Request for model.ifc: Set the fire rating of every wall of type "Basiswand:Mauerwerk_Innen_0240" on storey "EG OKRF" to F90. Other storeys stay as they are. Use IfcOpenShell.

First a look at what the model holds.

```python
import ifcopenshell
import ifcopenshell.util.element

model = ifcopenshell.open("model.ifc")
print(model.schema)
storey = next(s for s in model.by_type("IfcBuildingStorey") if s.Name == "EG OKRF")
walls = [e for e in ifcopenshell.util.element.get_decomposition(storey) if e.is_a("IfcWall")]
seen = {}
for e in walls:
    element_type = ifcopenshell.util.element.get_type(e)
    key = (element_type.Name if element_type != e and element_type else None, ifcopenshell.util.element.get_pset(e, "Pset_WallCommon", "FireRating"))
    seen[key] = seen.get(key, 0) + 1
for (name, value), count in sorted(seen.items(), key=str):
    print(count, "x", name, "|", value)
```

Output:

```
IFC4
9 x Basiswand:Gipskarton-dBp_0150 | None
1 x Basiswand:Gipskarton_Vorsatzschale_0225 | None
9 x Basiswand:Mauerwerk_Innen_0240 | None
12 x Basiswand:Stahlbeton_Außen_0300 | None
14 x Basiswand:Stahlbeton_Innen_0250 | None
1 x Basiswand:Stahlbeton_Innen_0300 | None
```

```python
import ifcopenshell
import ifcopenshell.api.pset
import ifcopenshell.util.element

model = ifcopenshell.open("model.ifc")

storey = next(s for s in model.by_type("IfcBuildingStorey") if s.Name == "EG OKRF")
walls = [e for e in ifcopenshell.util.element.get_decomposition(storey) if e.is_a("IfcWall")]

count = 0
for e in walls:
    element_type = ifcopenshell.util.element.get_type(e)
    if element_type in (None, e) or element_type.Name != "Basiswand:Mauerwerk_Innen_0240":
        continue
    # add_pset returns the element's existing set when there is one.
    pset = ifcopenshell.api.pset.add_pset(model, product=e, name="Pset_WallCommon")
    ifcopenshell.api.pset.edit_pset(model, pset=pset, properties={"FireRating": "F90"})
    count += 1

print(count, "walls updated")

model.write("model_updated.ifc")
```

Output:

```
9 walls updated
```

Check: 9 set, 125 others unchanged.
